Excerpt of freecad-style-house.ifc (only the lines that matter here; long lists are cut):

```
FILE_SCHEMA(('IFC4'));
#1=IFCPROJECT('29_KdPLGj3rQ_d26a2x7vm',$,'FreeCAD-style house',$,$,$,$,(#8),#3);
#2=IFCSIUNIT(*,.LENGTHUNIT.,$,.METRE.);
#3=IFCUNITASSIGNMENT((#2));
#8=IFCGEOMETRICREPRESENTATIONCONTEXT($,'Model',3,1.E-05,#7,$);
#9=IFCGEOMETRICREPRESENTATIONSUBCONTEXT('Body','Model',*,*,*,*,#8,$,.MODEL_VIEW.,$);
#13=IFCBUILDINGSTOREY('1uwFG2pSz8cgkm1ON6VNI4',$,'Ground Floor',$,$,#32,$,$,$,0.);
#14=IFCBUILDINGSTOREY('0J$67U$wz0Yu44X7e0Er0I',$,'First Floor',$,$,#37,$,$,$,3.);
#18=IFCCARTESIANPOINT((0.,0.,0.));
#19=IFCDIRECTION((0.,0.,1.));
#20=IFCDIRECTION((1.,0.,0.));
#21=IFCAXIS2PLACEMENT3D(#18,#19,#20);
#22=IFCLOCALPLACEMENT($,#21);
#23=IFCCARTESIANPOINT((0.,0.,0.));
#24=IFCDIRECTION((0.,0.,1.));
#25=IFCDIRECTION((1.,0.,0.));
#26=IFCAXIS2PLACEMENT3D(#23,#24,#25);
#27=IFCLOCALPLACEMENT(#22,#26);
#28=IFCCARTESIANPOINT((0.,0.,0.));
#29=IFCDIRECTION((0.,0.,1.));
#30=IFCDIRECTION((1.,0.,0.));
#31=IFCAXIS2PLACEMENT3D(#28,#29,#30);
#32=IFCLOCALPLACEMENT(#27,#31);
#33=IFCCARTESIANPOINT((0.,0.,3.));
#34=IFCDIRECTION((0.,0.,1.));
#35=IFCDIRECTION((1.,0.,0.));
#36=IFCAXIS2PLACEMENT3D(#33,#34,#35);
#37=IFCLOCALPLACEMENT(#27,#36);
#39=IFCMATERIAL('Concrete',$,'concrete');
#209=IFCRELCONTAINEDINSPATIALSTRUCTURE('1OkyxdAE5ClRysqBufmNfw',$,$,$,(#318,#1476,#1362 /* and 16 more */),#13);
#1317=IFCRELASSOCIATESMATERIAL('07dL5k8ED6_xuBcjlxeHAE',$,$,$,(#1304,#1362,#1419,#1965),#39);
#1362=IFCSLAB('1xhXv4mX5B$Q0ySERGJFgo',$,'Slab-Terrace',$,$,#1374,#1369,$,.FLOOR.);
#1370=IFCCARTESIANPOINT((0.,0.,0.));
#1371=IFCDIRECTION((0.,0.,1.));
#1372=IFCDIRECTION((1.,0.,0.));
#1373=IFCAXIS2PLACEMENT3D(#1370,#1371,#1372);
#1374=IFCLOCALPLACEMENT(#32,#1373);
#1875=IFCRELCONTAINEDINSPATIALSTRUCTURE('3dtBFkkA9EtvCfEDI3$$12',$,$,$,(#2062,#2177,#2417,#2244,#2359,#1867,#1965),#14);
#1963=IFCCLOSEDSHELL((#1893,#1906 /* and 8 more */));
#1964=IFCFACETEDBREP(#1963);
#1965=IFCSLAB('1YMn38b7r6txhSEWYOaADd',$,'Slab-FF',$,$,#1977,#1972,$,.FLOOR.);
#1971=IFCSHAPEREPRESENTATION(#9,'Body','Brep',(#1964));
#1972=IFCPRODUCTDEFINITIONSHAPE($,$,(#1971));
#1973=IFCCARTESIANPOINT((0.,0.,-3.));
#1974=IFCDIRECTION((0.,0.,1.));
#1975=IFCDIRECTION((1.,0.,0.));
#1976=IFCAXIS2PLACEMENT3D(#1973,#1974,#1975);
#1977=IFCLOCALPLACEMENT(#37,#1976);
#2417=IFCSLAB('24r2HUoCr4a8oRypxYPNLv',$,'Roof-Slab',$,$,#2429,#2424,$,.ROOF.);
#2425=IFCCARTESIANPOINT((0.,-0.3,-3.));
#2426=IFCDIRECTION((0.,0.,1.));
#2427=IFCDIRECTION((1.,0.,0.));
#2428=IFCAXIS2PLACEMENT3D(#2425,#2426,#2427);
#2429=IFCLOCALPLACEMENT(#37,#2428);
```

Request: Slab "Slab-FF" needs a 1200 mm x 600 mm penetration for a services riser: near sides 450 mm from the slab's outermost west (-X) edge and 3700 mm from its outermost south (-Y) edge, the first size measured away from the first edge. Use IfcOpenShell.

```python
import numpy as np
import ifcopenshell
import ifcopenshell.api.feature
import ifcopenshell.api.geometry
import ifcopenshell.api.root
import ifcopenshell.geom
import ifcopenshell.util.placement
import ifcopenshell.util.representation
import ifcopenshell.util.shape
import ifcopenshell.util.unit

model = ifcopenshell.open("freecad-style-house.ifc")
unit_scale = ifcopenshell.util.unit.calculate_unit_scale(model)
settings = ifcopenshell.geom.settings()


def volume(element):
    """Net volume in cubic metres, openings subtracted."""
    shape = ifcopenshell.geom.create_shape(settings, element)
    return ifcopenshell.util.shape.get_volume(shape.geometry)


slab = model.by_id(1965)
before = volume(slab)

# Extent in the slab's own axes, in metres. The edges named are its -X and -Y sides.
slab_shape = ifcopenshell.geom.create_shape(settings, slab)
vertices = ifcopenshell.util.shape.get_vertices(slab_shape.geometry)
x_min, y_min, bottom = vertices.min(axis=0)
top = vertices[:, 2].max()

opening = ifcopenshell.api.root.create_entity(model, ifc_class="IfcOpeningElement", name="Services riser opening", predefined_type="OPENING")
context = ifcopenshell.util.representation.get_context(model, "Model", "Body", "MODEL_VIEW")
width, depth = 1.2, 0.6
outline = [(0.0, 0.0), (width, 0.0), (width, depth), (0.0, depth), (0.0, 0.0)]
# Overshoot both faces by 50 mm so the cut is clean.
shape = ifcopenshell.api.geometry.add_slab_representation(
    model, context=context, depth=top - bottom + 0.1, polyline=outline
)
ifcopenshell.api.geometry.assign_representation(model, product=opening, representation=shape)

matrix = ifcopenshell.util.placement.get_local_placement(slab.ObjectPlacement)
matrix[:, 3] = matrix @ np.append(np.array([x_min + 0.45, y_min + 3.7, bottom - 0.05]) / unit_scale, 1.0)
ifcopenshell.api.geometry.edit_object_placement(model, product=opening, matrix=matrix, is_si=False)
ifcopenshell.api.feature.add_feature(model, feature=opening, element=slab)

after = volume(slab)

print(f"slab volume {before:.3f} -> {after:.3f} m3")

model.write("freecad-style-house_rev.ifc")
```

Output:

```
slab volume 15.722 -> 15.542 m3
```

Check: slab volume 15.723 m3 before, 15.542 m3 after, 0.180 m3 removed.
